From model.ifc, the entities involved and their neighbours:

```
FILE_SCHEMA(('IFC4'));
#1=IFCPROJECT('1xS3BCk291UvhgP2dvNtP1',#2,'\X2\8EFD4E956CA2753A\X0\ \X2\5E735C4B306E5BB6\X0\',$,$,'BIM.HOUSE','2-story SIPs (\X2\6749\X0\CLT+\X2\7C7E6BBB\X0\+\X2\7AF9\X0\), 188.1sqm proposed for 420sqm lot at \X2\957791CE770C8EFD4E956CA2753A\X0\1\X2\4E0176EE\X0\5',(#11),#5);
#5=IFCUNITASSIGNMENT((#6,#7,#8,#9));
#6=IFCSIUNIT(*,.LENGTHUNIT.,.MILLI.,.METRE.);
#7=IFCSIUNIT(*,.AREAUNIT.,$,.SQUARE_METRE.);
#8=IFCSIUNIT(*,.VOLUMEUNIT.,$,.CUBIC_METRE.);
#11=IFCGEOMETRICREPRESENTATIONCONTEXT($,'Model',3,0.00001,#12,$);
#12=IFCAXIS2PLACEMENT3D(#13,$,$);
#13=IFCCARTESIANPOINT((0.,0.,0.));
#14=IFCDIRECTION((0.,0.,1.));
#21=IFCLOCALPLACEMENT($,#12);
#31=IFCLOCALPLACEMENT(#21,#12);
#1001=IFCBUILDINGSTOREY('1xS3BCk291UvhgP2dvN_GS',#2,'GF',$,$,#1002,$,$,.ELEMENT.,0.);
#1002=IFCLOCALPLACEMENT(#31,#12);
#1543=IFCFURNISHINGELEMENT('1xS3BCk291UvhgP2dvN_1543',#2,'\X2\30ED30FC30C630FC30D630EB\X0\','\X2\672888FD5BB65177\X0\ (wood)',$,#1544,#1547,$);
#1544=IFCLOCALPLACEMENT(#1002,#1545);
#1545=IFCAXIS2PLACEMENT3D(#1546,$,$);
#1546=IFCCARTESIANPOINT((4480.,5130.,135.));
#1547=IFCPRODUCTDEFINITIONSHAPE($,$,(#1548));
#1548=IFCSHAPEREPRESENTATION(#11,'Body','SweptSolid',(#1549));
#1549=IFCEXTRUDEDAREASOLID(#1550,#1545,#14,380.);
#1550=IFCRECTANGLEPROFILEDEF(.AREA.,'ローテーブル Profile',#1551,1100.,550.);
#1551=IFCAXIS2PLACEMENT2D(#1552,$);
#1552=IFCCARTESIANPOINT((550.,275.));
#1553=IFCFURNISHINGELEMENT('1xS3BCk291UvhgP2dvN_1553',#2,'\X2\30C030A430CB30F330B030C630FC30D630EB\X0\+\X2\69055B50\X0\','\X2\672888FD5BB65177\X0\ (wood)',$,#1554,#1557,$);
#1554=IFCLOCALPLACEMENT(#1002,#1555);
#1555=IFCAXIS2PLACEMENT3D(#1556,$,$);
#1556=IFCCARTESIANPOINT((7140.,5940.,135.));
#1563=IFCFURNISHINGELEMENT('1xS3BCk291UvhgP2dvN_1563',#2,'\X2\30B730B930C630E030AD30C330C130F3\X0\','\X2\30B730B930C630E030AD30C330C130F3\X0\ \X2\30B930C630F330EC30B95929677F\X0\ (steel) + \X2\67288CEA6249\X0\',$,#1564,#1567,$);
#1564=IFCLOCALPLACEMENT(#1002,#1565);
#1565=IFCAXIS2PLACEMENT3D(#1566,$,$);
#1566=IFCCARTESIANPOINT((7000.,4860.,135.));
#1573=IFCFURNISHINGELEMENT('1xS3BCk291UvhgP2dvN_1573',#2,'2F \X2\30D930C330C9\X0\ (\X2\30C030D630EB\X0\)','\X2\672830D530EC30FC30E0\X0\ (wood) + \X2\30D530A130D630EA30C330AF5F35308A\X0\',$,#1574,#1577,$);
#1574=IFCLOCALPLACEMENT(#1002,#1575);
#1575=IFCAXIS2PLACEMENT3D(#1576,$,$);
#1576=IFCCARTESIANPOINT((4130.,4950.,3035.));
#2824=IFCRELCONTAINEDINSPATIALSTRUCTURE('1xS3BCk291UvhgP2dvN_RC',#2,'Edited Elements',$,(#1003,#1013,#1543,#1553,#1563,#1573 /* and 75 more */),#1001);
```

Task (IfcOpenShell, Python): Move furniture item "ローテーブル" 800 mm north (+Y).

```python
import ifcopenshell
import ifcopenshell.api.geometry
import ifcopenshell.util.placement
import ifcopenshell.util.unit

model = ifcopenshell.open("model.ifc")
unit_scale = ifcopenshell.util.unit.calculate_unit_scale(model)

item = model.by_guid("1xS3BCk291UvhgP2dvN_1543")
matrix = ifcopenshell.util.placement.get_local_placement(item.ObjectPlacement)
matrix[1, 3] += 0.8 / unit_scale
ifcopenshell.api.geometry.edit_object_placement(model, product=item, matrix=matrix, is_si=False)

print(ifcopenshell.util.placement.get_local_placement(item.ObjectPlacement).round(3) + 0.0)

model.write("model_updated.ifc")
```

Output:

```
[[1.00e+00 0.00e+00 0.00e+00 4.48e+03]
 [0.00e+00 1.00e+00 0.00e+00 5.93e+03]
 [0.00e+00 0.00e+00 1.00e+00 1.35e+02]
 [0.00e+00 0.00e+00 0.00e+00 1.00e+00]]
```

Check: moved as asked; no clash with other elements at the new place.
